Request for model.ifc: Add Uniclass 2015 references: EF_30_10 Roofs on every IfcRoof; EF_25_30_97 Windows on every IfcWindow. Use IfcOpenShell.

First a look at what the model holds.

```python
import ifcopenshell

model = ifcopenshell.open("model.ifc")
print(model.schema)
print("classifications:", [c.Name for c in model.by_type("IfcClassification")])
for ifc_class in ("IfcDoor", "IfcRoof", "IfcStair", "IfcWall", "IfcWindow"):
    print(ifc_class, len(model.by_type(ifc_class)))
```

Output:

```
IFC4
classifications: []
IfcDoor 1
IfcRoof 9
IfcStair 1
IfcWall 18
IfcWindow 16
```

```python
import ifcopenshell
import ifcopenshell.api.classification

model = ifcopenshell.open("model.ifc")

system = ifcopenshell.api.classification.add_classification(model, classification="Uniclass 2015")

codes = {
    "IfcRoof": ("EF_30_10", "Roofs"),
    "IfcWindow": ("EF_25_30_97", "Windows"),
}
for ifc_class, (code, name) in codes.items():
    products = model.by_type(ifc_class)
    ifcopenshell.api.classification.add_reference(
        model, products=products, classification=system, identification=code, name=name
    )
    print(code, len(products))

model.write("model_v2.ifc")
```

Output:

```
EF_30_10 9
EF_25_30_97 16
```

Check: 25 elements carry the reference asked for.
